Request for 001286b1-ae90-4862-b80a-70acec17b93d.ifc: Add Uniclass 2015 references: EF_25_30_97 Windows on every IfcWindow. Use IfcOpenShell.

First a look at what the model holds.

```python
import ifcopenshell

model = ifcopenshell.open("001286b1-ae90-4862-b80a-70acec17b93d.ifc")
print(model.schema)
print("classifications:", [c.Name for c in model.by_type("IfcClassification")])
for ifc_class in ("IfcDoor", "IfcRoof", "IfcStair", "IfcWall", "IfcWindow"):
    print(ifc_class, len(model.by_type(ifc_class)))
```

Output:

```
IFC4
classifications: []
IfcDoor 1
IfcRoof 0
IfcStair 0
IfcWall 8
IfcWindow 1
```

```python
import ifcopenshell
import ifcopenshell.api.classification

model = ifcopenshell.open("001286b1-ae90-4862-b80a-70acec17b93d.ifc")

system = ifcopenshell.api.classification.add_classification(model, classification="Uniclass 2015")

codes = {
    "IfcWindow": ("EF_25_30_97", "Windows"),
}
for ifc_class, (code, name) in codes.items():
    products = model.by_type(ifc_class)
    ifcopenshell.api.classification.add_reference(
        model, products=products, classification=system, identification=code, name=name
    )
    print(code, len(products))

model.write("001286b1-ae90-4862-b80a-70acec17b93d_updated.ifc")
```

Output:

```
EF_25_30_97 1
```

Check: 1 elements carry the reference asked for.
